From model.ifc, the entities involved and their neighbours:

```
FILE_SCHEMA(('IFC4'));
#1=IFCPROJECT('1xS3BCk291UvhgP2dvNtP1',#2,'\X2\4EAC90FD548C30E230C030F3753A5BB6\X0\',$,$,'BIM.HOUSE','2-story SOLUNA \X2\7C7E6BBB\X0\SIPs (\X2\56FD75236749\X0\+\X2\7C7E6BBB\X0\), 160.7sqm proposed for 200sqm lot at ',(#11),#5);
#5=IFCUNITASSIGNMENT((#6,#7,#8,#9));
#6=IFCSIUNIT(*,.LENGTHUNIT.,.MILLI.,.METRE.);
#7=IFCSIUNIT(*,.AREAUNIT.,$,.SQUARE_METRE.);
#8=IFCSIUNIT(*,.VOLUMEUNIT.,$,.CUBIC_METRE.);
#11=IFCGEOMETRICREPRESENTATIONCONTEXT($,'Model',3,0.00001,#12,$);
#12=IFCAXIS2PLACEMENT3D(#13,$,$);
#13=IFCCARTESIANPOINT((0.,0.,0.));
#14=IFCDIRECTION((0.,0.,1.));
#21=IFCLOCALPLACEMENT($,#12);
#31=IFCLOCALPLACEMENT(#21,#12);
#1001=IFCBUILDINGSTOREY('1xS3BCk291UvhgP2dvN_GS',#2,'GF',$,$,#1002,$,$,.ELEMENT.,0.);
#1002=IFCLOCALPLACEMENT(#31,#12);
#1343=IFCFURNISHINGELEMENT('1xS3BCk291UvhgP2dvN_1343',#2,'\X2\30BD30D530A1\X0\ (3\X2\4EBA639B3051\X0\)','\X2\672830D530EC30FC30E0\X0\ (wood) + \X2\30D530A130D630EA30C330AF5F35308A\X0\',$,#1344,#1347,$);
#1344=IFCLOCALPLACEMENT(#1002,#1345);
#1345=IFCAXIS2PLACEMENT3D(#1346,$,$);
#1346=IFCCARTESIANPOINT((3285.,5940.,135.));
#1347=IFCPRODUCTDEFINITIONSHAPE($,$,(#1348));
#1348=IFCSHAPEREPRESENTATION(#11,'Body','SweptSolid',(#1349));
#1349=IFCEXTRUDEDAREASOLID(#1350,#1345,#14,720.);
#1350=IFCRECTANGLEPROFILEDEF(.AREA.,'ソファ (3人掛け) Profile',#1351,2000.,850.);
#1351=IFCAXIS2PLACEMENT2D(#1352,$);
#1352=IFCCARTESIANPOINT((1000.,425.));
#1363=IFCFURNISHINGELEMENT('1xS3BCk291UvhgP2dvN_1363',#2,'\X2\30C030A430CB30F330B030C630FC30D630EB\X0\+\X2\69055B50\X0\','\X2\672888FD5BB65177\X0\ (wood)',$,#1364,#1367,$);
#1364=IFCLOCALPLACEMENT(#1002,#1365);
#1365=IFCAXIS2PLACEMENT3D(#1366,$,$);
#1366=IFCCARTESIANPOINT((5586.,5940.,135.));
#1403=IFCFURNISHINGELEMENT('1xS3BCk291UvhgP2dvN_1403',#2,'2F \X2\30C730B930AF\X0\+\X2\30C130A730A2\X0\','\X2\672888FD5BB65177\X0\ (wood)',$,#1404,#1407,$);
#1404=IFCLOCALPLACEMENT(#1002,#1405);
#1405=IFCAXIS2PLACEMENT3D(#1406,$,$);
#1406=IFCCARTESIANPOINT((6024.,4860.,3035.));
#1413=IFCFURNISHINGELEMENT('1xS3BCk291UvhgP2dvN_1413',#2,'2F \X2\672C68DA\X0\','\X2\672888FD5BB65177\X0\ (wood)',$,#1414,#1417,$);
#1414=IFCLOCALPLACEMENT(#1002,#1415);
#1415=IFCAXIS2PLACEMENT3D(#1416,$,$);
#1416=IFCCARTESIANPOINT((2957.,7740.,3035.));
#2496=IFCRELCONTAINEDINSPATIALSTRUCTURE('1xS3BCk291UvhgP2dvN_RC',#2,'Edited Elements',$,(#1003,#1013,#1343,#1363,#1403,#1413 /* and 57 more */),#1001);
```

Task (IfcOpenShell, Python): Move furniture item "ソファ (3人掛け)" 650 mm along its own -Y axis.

```python
import ifcopenshell
import ifcopenshell.api.geometry
import ifcopenshell.util.placement

model = ifcopenshell.open("model.ifc")

item = model.by_guid("1xS3BCk291UvhgP2dvN_1343")
matrix = ifcopenshell.util.placement.get_local_placement(item.ObjectPlacement)
matrix[:3, 3] -= matrix[:3, 1] * 650.0
ifcopenshell.api.geometry.edit_object_placement(model, product=item, matrix=matrix, is_si=False)

print(ifcopenshell.util.placement.get_local_placement(item.ObjectPlacement).round(3) + 0.0)

model.write("model-out.ifc")
```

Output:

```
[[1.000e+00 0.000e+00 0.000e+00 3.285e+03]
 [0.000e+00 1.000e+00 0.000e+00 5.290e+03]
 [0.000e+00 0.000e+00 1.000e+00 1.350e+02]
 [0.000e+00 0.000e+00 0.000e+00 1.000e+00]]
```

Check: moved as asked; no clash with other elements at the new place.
